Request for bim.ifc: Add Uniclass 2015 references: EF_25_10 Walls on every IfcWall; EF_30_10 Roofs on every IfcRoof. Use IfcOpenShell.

First a look at what the model holds.

```python
import ifcopenshell

model = ifcopenshell.open("bim.ifc")
print(model.schema)
print("classifications:", [c.Name for c in model.by_type("IfcClassification")])
for ifc_class in ("IfcDoor", "IfcRoof", "IfcStair", "IfcWall", "IfcWindow"):
    print(ifc_class, len(model.by_type(ifc_class)))
```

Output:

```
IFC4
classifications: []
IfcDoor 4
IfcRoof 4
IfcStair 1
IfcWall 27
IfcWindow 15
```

```python
import ifcopenshell
import ifcopenshell.api.classification

model = ifcopenshell.open("bim.ifc")

system = ifcopenshell.api.classification.add_classification(model, classification="Uniclass 2015")

codes = {
    "IfcWall": ("EF_25_10", "Walls"),
    "IfcRoof": ("EF_30_10", "Roofs"),
}
for ifc_class, (code, name) in codes.items():
    products = model.by_type(ifc_class)
    ifcopenshell.api.classification.add_reference(
        model, products=products, classification=system, identification=code, name=name
    )
    print(code, len(products))

model.write("bim_rev.ifc")
```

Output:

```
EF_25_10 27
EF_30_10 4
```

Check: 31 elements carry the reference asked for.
